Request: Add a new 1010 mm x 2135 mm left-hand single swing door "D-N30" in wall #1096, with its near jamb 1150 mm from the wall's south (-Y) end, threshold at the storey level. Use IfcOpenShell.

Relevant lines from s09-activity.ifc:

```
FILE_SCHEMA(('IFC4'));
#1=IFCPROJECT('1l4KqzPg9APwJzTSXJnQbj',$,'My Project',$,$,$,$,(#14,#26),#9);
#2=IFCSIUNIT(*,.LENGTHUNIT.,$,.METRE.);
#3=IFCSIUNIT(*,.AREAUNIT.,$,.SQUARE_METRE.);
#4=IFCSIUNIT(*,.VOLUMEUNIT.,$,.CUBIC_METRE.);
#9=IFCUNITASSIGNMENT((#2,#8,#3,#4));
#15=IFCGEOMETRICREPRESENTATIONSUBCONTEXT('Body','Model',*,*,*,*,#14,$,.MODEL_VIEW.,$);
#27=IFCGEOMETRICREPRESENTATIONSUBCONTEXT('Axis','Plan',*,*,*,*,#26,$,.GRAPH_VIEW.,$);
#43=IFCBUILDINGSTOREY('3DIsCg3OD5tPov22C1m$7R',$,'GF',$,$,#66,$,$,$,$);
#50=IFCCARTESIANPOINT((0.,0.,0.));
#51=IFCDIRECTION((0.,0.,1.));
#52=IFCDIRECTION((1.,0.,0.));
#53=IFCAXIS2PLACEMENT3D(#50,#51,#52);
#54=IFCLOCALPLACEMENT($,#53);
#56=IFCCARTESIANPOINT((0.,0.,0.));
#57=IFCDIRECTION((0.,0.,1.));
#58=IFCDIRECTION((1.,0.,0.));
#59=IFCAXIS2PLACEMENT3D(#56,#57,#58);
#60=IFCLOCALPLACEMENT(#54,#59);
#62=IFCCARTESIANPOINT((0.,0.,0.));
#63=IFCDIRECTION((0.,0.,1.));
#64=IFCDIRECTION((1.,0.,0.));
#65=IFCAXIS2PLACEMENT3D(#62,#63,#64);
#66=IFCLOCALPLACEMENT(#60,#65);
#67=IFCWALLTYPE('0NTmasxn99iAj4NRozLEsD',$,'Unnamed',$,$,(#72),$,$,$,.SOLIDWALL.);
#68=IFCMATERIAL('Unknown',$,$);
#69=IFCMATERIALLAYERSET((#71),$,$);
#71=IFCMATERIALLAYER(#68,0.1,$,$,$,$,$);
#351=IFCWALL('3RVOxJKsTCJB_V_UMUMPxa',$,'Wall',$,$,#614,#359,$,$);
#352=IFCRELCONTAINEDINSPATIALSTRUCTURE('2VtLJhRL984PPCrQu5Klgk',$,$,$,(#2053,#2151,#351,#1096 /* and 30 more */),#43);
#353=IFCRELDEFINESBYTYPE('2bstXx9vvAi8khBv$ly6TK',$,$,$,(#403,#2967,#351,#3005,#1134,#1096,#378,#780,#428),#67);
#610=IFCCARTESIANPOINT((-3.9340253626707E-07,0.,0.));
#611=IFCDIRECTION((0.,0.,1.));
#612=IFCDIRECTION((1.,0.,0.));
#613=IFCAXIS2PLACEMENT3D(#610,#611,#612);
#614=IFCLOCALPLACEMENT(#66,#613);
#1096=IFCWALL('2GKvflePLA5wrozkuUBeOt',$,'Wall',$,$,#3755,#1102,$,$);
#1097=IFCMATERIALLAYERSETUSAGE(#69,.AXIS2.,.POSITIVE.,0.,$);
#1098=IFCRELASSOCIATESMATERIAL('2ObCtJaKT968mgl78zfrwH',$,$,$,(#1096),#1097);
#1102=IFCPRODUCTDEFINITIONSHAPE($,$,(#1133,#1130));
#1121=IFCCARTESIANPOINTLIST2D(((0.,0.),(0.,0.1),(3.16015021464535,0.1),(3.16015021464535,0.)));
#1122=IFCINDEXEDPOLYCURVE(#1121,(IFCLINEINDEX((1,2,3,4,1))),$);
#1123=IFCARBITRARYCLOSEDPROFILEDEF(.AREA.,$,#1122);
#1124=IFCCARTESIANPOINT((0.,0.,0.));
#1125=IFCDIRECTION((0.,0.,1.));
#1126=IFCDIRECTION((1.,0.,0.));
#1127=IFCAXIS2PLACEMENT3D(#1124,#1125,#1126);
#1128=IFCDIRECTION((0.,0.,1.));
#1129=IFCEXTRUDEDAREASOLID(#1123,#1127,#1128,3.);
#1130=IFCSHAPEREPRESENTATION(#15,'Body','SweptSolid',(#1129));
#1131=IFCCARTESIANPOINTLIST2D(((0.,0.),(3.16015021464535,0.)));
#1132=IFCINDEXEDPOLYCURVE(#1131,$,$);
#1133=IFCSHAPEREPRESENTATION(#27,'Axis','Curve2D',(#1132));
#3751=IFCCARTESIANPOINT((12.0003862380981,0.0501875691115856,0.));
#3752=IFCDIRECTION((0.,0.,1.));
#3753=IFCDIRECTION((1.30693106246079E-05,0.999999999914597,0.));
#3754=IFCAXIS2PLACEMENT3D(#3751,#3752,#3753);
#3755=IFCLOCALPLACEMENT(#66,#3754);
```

```python
import numpy as np
import ifcopenshell
import ifcopenshell.api.feature
import ifcopenshell.api.geometry
import ifcopenshell.api.root
import ifcopenshell.api.spatial
import ifcopenshell.geom
import ifcopenshell.util.element
import ifcopenshell.util.placement
import ifcopenshell.util.representation
import ifcopenshell.util.shape
import ifcopenshell.util.unit

model = ifcopenshell.open("s09-activity.ifc")
unit_scale = ifcopenshell.util.unit.calculate_unit_scale(model)
settings = ifcopenshell.geom.settings()


def volume(element):
    """Net volume in cubic metres, openings subtracted."""
    shape = ifcopenshell.geom.create_shape(settings, element)
    return ifcopenshell.util.shape.get_volume(shape.geometry)


wall = model.by_guid("2GKvflePLA5wrozkuUBeOt")
storey = ifcopenshell.util.element.get_container(wall, ifc_class="IfcBuildingStorey")
context = ifcopenshell.util.representation.get_context(model, "Model", "Body", "MODEL_VIEW")
before = volume(wall)

width, height, from_end, sill = 1.01, 2.135, 1.15, 0.0  # metres

# The wall runs along its own X axis, and the end named is its -X end.
wall_shape = ifcopenshell.geom.create_shape(settings, wall)
x, y, z = ifcopenshell.util.shape.get_vertices(wall_shape.geometry).T
start = x.min() + from_end
face, thickness = float(y.min()), float(y.max() - y.min())
wall_matrix = ifcopenshell.util.placement.get_local_placement(wall.ObjectPlacement)
level = ifcopenshell.util.placement.get_local_placement(storey.ObjectPlacement)[2, 3]


def in_wall(x, y):
    """Placement at x, y metres in the wall's axes, at sill height."""
    matrix = wall_matrix.copy()
    matrix[:, 3] = wall_matrix @ np.array([x / unit_scale, y / unit_scale, 0.0, 1.0])
    matrix[2, 3] = level + sill / unit_scale
    return matrix


# Opening: a box that overshoots both wall faces by 50 mm.
opening = ifcopenshell.api.root.create_entity(model, ifc_class="IfcOpeningElement", predefined_type="OPENING")
box = ifcopenshell.api.geometry.add_wall_representation(
    model, context=context, length=width, height=height, thickness=thickness + 0.1
)
ifcopenshell.api.geometry.assign_representation(model, product=opening, representation=box)
ifcopenshell.api.geometry.edit_object_placement(model, product=opening, matrix=in_wall(start, face - 0.05), is_si=False)
ifcopenshell.api.feature.add_feature(model, feature=opening, element=wall)

door = ifcopenshell.api.root.create_entity(model, ifc_class="IfcDoor", name="D-N30", predefined_type="DOOR")
door.OverallWidth, door.OverallHeight = width / unit_scale, height / unit_scale
door.OperationType = "SINGLE_SWING_LEFT"
body = ifcopenshell.api.geometry.add_door_representation(
    model,
    context=context,
    overall_width=door.OverallWidth,
    overall_height=door.OverallHeight,
    operation_type="SINGLE_SWING_LEFT",
    lining_properties={"LiningDepth": thickness / unit_scale, "ThresholdDepth": thickness / unit_scale},
)
ifcopenshell.api.geometry.assign_representation(model, product=door, representation=body)
ifcopenshell.api.spatial.assign_container(model, products=[door], relating_structure=storey)
ifcopenshell.api.feature.add_filling(model, opening=opening, element=door)

# The lining spans the wall, so the door starts at the wall face.
ifcopenshell.api.geometry.edit_object_placement(model, product=door, matrix=in_wall(start, face), is_si=False)

after = volume(wall)

print(f"wall volume {before:.3f} -> {after:.3f} m3")

model.write("s09-activity-out.ifc")
```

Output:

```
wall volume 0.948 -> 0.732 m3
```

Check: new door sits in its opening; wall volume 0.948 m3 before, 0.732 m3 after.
